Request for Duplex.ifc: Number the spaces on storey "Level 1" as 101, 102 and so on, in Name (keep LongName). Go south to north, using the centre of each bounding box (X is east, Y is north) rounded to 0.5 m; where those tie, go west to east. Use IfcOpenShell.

First a look at what the model holds.

```python
import ifcopenshell
import ifcopenshell.util.element
import ifcopenshell.util.placement

model = ifcopenshell.open("Duplex.ifc")
print(model.schema)
storey = next(s for s in model.by_type("IfcBuildingStorey") if s.Name == "Level 1")
spaces = [e for e in ifcopenshell.util.element.get_decomposition(storey) if e.is_a("IfcSpace")]
for e in sorted(spaces, key=lambda e: e.id()):
    origin = ifcopenshell.util.placement.get_local_placement(e.ObjectPlacement)[:3, 3]
    print(e.id(), e.Name, e.LongName, origin.round(2) + 0.0, sep=" | ")
```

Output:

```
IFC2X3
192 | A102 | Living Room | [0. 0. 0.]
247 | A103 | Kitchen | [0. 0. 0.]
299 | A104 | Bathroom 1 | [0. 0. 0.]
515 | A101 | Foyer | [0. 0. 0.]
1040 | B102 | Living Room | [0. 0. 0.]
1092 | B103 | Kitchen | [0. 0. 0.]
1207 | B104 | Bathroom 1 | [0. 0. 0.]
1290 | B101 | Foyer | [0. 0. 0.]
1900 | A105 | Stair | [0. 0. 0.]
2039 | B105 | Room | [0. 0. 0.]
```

```python
import ifcopenshell
import ifcopenshell.geom
import ifcopenshell.util.element
import ifcopenshell.util.shape

model = ifcopenshell.open("Duplex.ifc")
settings = ifcopenshell.geom.settings()
settings.set("use-world-coords", True)


def centre(element):
    shape = ifcopenshell.geom.create_shape(settings, element)
    return ifcopenshell.util.shape.get_bbox_centroid(shape.geometry)


storey = next(s for s in model.by_type("IfcBuildingStorey") if s.Name == "Level 1")
spaces = [e for e in ifcopenshell.util.element.get_decomposition(storey) if e.is_a("IfcSpace")]

# Insertion points can sit at a corner or the storey origin, so sort by the geometry (in metres).
centres = {e: centre(e) for e in spaces}
spaces.sort(key=lambda e: (round(centres[e][1] / 0.5), centres[e][0]))

for i, e in enumerate(spaces, start=1):
    number = f"1{i:02d}"
    e.Name = number
    print(e.id(), number)

model.write("Duplex-out.ifc")
```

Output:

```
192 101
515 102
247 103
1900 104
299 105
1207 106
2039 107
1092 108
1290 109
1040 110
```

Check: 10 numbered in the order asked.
